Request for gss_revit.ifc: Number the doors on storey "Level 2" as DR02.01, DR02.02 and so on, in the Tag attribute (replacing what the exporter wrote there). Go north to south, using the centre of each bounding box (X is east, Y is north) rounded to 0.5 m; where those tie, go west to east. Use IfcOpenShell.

First a look at what the model holds.

```python
import ifcopenshell
import ifcopenshell.util.element
import ifcopenshell.util.placement

model = ifcopenshell.open("gss_revit.ifc")
print(model.schema)
storey = next(s for s in model.by_type("IfcBuildingStorey") if s.Name == "Level 2")
doors = [e for e in ifcopenshell.util.element.get_decomposition(storey) if e.is_a("IfcDoor")]
for e in sorted(doors, key=lambda e: e.id()):
    origin = ifcopenshell.util.placement.get_local_placement(e.ObjectPlacement)[:3, 3]
    print(e.id(), e.Tag, e.Name, origin.round(2) + 0.0, sep=" | ")
```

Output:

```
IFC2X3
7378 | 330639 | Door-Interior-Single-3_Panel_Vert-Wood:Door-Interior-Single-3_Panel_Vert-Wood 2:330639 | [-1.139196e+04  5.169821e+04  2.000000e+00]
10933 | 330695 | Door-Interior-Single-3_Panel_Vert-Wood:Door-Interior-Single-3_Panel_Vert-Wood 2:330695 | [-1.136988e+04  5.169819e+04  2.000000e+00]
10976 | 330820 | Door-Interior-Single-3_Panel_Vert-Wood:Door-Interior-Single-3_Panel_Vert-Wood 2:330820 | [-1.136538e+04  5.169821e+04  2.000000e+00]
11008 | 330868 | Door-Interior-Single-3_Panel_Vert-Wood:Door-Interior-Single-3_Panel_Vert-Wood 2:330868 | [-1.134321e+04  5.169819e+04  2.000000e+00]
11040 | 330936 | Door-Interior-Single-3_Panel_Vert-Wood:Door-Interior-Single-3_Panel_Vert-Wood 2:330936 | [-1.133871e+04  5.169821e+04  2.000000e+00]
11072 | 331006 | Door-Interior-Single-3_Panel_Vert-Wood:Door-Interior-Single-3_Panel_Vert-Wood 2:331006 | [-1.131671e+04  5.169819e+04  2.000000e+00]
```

```python
import ifcopenshell
import ifcopenshell.geom
import ifcopenshell.util.element
import ifcopenshell.util.shape

model = ifcopenshell.open("gss_revit.ifc")
settings = ifcopenshell.geom.settings()
settings.set("use-world-coords", True)


def centre(element):
    shape = ifcopenshell.geom.create_shape(settings, element)
    return ifcopenshell.util.shape.get_bbox_centroid(shape.geometry)


storey = next(s for s in model.by_type("IfcBuildingStorey") if s.Name == "Level 2")
doors = [e for e in ifcopenshell.util.element.get_decomposition(storey) if e.is_a("IfcDoor")]

# Insertion points can sit at a corner or the storey origin, so sort by the geometry (in metres).
centres = {e: centre(e) for e in doors}
doors.sort(key=lambda e: (-round(centres[e][1] / 0.5), centres[e][0]))

for i, e in enumerate(doors, start=1):
    number = f"DR02.{i:02d}"
    e.Tag = number
    print(e.id(), number)

model.write("gss_revit_edited.ifc")
```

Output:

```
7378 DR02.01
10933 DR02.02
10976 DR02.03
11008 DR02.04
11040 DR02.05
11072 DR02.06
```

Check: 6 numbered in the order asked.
